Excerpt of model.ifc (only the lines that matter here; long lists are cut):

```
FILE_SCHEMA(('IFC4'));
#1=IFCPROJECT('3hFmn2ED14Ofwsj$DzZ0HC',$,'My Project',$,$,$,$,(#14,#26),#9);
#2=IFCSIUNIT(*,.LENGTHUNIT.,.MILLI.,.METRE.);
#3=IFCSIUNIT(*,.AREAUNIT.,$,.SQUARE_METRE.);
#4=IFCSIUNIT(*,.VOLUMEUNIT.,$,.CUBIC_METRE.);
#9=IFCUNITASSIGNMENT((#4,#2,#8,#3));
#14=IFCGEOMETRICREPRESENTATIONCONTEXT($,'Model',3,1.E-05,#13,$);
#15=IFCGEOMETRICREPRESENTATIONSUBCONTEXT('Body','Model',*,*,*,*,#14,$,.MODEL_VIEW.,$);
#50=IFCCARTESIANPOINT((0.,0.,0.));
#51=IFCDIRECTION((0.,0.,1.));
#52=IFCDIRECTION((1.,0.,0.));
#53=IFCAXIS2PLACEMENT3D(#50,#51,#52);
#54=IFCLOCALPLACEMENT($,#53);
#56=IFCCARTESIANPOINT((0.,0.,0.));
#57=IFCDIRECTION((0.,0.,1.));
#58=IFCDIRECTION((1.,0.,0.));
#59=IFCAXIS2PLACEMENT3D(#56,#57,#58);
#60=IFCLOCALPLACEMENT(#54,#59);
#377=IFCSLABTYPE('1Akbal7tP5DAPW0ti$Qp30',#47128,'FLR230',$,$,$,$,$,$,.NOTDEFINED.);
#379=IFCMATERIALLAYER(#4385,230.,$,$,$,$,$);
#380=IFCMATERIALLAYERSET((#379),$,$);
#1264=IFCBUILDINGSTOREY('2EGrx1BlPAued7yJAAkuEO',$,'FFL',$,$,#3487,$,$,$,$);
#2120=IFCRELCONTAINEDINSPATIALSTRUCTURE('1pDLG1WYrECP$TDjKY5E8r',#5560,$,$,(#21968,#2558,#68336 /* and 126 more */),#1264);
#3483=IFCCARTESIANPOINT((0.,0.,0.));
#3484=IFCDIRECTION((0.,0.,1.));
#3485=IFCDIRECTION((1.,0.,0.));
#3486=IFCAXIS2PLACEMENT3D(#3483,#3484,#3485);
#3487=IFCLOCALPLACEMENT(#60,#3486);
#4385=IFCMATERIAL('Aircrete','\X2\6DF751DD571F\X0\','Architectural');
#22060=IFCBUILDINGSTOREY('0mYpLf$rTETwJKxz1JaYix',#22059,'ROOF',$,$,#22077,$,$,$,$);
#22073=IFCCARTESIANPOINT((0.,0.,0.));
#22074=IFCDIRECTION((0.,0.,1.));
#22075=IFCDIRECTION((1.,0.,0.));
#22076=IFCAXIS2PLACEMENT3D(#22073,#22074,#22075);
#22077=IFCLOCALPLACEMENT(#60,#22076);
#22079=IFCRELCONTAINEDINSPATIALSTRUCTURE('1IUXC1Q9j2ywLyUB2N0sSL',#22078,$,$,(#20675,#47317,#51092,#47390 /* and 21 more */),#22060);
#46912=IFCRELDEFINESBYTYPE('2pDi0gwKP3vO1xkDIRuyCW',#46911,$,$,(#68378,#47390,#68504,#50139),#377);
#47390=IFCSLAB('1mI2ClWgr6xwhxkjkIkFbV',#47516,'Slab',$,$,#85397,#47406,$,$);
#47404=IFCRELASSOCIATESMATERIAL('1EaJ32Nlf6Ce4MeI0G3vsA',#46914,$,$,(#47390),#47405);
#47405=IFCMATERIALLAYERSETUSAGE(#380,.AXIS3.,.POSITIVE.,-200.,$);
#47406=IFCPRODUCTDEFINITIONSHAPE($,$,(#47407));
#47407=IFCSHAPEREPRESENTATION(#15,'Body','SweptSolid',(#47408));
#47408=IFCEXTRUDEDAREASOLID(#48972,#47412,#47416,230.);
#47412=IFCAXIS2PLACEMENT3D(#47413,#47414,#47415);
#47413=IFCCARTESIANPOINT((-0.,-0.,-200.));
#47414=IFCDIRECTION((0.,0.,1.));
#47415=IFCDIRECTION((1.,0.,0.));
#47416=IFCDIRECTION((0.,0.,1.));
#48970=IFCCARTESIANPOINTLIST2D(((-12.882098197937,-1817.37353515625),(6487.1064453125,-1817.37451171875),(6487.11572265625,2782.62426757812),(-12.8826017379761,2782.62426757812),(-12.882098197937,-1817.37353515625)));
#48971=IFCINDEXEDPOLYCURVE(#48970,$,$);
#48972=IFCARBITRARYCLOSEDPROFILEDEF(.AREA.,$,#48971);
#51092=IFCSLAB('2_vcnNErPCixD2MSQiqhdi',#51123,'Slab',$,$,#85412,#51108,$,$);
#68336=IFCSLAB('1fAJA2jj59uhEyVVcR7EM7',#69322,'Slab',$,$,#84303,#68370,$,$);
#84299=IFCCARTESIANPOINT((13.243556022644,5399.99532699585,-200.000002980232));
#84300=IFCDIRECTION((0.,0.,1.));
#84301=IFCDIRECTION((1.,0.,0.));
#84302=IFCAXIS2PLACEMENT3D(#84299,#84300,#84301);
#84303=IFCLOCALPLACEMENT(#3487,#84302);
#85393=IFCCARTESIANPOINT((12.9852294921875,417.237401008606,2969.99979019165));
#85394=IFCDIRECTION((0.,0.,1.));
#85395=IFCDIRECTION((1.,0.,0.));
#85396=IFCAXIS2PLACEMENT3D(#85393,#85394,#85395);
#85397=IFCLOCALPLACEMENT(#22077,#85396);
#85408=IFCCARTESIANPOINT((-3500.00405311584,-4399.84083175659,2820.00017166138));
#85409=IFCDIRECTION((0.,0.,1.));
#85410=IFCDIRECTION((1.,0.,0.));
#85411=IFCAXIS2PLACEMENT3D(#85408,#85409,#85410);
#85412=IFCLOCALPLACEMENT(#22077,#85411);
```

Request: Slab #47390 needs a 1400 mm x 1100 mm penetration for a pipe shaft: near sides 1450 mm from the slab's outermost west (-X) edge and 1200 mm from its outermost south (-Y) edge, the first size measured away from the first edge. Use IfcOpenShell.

```python
import numpy as np
import ifcopenshell
import ifcopenshell.api.feature
import ifcopenshell.api.geometry
import ifcopenshell.api.root
import ifcopenshell.geom
import ifcopenshell.util.placement
import ifcopenshell.util.representation
import ifcopenshell.util.shape
import ifcopenshell.util.unit

model = ifcopenshell.open("model.ifc")
unit_scale = ifcopenshell.util.unit.calculate_unit_scale(model)
settings = ifcopenshell.geom.settings()


def volume(element):
    """Net volume in cubic metres, openings subtracted."""
    shape = ifcopenshell.geom.create_shape(settings, element)
    return ifcopenshell.util.shape.get_volume(shape.geometry)


slab = model.by_id(47390)
before = volume(slab)

# Extent in the slab's own axes, in metres. The edges named are its -X and -Y sides.
slab_shape = ifcopenshell.geom.create_shape(settings, slab)
vertices = ifcopenshell.util.shape.get_vertices(slab_shape.geometry)
x_min, y_min, bottom = vertices.min(axis=0)
top = vertices[:, 2].max()

opening = ifcopenshell.api.root.create_entity(model, ifc_class="IfcOpeningElement", name="Pipe shaft opening", predefined_type="OPENING")
context = ifcopenshell.util.representation.get_context(model, "Model", "Body", "MODEL_VIEW")
width, depth = 1.4, 1.1
outline = [(0.0, 0.0), (width, 0.0), (width, depth), (0.0, depth), (0.0, 0.0)]
# Overshoot both faces by 50 mm so the cut is clean.
shape = ifcopenshell.api.geometry.add_slab_representation(
    model, context=context, depth=top - bottom + 0.1, polyline=outline
)
ifcopenshell.api.geometry.assign_representation(model, product=opening, representation=shape)

matrix = ifcopenshell.util.placement.get_local_placement(slab.ObjectPlacement)
matrix[:, 3] = matrix @ np.append(np.array([x_min + 1.45, y_min + 1.2, bottom - 0.05]) / unit_scale, 1.0)
ifcopenshell.api.geometry.edit_object_placement(model, product=opening, matrix=matrix, is_si=False)
ifcopenshell.api.feature.add_feature(model, feature=opening, element=slab)

after = volume(slab)

print(f"slab volume {before:.3f} -> {after:.3f} m3")

model.write("model_edited.ifc")
```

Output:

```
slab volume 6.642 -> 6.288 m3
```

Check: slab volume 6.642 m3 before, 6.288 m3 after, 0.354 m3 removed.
